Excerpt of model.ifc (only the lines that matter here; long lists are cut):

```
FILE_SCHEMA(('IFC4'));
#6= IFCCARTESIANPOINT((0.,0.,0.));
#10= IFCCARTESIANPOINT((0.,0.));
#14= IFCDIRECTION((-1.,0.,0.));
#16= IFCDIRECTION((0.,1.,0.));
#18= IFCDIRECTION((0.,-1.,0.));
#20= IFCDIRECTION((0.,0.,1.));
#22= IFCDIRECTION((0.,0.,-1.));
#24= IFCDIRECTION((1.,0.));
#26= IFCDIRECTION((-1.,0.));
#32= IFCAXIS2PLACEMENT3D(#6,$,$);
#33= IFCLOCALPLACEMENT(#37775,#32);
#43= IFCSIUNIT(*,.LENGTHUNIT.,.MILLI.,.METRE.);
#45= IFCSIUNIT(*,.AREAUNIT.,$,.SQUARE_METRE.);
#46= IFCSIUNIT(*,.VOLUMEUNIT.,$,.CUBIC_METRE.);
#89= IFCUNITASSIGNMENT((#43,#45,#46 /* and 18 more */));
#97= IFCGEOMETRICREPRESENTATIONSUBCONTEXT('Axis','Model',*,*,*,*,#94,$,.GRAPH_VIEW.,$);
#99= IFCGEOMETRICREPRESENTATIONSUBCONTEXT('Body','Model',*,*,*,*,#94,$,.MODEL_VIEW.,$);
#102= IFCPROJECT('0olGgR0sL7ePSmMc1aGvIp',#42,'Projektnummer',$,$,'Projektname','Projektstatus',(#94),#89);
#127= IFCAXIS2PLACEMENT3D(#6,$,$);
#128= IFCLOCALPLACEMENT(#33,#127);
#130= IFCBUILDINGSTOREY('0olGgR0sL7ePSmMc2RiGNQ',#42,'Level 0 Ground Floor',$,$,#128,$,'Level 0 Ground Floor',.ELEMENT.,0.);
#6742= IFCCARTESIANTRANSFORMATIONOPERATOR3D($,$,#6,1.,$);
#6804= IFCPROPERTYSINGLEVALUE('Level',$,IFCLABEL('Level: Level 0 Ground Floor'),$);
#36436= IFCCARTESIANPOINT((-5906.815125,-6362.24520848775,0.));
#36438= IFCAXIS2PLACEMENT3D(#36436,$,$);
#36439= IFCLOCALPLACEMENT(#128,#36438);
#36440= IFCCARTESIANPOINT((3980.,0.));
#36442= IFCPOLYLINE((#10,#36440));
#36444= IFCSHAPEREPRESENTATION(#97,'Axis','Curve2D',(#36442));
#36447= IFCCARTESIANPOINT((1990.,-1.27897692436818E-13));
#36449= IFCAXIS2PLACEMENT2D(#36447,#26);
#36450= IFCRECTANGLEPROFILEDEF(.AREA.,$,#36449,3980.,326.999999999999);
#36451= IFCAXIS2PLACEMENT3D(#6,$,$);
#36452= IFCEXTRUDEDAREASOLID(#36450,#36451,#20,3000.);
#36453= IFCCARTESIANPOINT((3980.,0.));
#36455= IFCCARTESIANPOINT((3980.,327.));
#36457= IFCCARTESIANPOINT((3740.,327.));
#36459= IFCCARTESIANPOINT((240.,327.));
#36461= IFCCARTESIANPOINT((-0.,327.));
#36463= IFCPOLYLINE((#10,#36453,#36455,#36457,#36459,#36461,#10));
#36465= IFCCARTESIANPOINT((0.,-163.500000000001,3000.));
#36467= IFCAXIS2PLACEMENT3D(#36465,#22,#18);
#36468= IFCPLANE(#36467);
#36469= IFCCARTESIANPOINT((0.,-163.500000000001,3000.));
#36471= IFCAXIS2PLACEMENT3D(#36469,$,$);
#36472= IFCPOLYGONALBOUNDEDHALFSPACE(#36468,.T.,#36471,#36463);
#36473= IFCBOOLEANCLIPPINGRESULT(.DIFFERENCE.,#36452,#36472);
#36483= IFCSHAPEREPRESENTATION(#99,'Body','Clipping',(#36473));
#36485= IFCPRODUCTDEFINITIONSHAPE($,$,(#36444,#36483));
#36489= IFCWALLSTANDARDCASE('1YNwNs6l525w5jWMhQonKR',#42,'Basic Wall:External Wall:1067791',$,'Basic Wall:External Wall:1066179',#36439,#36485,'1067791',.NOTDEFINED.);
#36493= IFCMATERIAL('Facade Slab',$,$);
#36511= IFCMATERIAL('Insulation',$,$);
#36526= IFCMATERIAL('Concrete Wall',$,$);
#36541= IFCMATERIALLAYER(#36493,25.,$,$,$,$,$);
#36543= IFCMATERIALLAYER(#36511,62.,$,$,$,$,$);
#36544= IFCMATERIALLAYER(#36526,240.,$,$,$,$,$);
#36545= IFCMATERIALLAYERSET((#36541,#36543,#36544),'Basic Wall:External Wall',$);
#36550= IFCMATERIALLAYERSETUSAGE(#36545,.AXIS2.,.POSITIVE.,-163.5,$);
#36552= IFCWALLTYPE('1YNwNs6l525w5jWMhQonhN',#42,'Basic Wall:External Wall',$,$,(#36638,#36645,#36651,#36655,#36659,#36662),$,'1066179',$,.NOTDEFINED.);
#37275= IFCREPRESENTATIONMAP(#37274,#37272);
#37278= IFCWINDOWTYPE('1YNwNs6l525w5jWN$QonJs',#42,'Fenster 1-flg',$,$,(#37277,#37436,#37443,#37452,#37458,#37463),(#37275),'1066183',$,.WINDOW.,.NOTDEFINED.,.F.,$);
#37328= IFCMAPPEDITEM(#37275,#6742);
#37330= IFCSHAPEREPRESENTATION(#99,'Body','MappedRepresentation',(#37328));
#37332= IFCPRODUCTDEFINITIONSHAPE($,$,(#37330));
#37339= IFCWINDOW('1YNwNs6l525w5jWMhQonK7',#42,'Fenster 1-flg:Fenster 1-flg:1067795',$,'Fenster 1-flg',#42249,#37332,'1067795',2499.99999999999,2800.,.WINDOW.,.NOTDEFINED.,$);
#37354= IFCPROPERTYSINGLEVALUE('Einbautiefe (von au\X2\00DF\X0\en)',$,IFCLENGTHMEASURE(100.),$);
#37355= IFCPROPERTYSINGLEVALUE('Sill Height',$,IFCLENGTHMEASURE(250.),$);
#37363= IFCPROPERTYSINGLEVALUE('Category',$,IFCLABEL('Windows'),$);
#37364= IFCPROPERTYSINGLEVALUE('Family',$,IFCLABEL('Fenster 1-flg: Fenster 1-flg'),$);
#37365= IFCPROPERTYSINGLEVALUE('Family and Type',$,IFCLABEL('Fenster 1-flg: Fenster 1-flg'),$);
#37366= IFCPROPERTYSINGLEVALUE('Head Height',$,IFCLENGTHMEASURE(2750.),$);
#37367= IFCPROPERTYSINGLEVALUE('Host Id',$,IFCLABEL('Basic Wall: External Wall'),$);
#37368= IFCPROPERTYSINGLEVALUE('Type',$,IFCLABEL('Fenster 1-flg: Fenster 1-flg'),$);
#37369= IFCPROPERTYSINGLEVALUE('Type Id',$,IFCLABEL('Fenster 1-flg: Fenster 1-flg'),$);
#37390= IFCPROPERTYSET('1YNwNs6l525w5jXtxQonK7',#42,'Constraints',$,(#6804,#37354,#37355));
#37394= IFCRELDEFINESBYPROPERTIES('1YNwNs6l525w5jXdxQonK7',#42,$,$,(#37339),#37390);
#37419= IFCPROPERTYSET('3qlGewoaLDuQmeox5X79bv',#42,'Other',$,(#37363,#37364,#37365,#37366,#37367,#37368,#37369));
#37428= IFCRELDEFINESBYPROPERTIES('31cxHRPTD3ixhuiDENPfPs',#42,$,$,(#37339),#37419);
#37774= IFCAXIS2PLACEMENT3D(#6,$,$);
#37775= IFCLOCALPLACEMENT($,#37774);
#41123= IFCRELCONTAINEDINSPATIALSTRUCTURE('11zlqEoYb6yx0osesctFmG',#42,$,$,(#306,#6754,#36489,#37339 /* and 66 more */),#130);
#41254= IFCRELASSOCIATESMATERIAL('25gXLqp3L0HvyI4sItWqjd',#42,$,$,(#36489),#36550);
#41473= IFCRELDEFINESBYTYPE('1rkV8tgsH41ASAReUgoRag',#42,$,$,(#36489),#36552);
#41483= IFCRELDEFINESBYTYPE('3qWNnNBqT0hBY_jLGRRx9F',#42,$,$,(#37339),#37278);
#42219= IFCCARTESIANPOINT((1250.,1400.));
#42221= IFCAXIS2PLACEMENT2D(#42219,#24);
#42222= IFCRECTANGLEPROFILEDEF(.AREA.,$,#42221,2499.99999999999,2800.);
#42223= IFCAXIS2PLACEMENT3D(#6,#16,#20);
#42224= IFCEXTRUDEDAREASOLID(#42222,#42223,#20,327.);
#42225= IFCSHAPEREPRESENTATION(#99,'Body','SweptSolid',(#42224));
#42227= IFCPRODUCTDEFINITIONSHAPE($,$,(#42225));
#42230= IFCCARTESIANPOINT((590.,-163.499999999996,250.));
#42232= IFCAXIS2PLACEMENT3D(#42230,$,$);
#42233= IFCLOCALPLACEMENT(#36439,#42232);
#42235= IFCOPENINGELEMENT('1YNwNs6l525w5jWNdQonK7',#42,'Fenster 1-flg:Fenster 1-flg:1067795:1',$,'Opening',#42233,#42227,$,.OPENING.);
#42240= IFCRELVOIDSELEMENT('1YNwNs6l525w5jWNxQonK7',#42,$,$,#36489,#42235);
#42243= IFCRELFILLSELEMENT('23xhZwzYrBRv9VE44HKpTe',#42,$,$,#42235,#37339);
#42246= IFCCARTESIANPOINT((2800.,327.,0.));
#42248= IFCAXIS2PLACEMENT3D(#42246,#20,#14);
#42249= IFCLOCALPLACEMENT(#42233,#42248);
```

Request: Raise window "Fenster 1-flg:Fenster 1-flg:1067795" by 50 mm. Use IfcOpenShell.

```python
import numpy as np
import ifcopenshell
import ifcopenshell.api.geometry
import ifcopenshell.api.pset
import ifcopenshell.util.element
import ifcopenshell.util.placement
import ifcopenshell.util.unit

model = ifcopenshell.open("model.ifc")
unit_scale = ifcopenshell.util.unit.calculate_unit_scale(model)

window = model.by_guid("1YNwNs6l525w5jWMhQonK7")
opening = window.FillsVoids[0].RelatingOpeningElement
dz = 0.05 / unit_scale

shift = np.array([0.0, 0.0, dz])
# The window is placed relative to its opening, so it follows when the opening moves.
matrix = ifcopenshell.util.placement.get_local_placement(opening.ObjectPlacement)
matrix[:3, 3] += shift
ifcopenshell.api.geometry.edit_object_placement(
    model, product=opening, matrix=matrix, is_si=False, should_transform_children=True
)

# Keep the stored heights in step.
pset = model.by_id(ifcopenshell.util.element.get_pset(window, "Constraints", should_inherit=False)["id"])
ifcopenshell.api.pset.edit_pset(model, pset=pset, properties={
    "Sill Height": model.create_entity("IfcLengthMeasure", ifcopenshell.util.element.get_pset(window, "Constraints", "Sill Height") + dz),
})
pset = model.by_id(ifcopenshell.util.element.get_pset(window, "Other", should_inherit=False)["id"])
ifcopenshell.api.pset.edit_pset(model, pset=pset, properties={
    "Head Height": model.create_entity("IfcLengthMeasure", ifcopenshell.util.element.get_pset(window, "Other", "Head Height") + dz),
})

print(f"moved by {dz * unit_scale:+.3f} m")

model.write("model_updated.ifc")
```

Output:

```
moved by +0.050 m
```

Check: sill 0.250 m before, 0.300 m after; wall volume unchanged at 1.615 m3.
